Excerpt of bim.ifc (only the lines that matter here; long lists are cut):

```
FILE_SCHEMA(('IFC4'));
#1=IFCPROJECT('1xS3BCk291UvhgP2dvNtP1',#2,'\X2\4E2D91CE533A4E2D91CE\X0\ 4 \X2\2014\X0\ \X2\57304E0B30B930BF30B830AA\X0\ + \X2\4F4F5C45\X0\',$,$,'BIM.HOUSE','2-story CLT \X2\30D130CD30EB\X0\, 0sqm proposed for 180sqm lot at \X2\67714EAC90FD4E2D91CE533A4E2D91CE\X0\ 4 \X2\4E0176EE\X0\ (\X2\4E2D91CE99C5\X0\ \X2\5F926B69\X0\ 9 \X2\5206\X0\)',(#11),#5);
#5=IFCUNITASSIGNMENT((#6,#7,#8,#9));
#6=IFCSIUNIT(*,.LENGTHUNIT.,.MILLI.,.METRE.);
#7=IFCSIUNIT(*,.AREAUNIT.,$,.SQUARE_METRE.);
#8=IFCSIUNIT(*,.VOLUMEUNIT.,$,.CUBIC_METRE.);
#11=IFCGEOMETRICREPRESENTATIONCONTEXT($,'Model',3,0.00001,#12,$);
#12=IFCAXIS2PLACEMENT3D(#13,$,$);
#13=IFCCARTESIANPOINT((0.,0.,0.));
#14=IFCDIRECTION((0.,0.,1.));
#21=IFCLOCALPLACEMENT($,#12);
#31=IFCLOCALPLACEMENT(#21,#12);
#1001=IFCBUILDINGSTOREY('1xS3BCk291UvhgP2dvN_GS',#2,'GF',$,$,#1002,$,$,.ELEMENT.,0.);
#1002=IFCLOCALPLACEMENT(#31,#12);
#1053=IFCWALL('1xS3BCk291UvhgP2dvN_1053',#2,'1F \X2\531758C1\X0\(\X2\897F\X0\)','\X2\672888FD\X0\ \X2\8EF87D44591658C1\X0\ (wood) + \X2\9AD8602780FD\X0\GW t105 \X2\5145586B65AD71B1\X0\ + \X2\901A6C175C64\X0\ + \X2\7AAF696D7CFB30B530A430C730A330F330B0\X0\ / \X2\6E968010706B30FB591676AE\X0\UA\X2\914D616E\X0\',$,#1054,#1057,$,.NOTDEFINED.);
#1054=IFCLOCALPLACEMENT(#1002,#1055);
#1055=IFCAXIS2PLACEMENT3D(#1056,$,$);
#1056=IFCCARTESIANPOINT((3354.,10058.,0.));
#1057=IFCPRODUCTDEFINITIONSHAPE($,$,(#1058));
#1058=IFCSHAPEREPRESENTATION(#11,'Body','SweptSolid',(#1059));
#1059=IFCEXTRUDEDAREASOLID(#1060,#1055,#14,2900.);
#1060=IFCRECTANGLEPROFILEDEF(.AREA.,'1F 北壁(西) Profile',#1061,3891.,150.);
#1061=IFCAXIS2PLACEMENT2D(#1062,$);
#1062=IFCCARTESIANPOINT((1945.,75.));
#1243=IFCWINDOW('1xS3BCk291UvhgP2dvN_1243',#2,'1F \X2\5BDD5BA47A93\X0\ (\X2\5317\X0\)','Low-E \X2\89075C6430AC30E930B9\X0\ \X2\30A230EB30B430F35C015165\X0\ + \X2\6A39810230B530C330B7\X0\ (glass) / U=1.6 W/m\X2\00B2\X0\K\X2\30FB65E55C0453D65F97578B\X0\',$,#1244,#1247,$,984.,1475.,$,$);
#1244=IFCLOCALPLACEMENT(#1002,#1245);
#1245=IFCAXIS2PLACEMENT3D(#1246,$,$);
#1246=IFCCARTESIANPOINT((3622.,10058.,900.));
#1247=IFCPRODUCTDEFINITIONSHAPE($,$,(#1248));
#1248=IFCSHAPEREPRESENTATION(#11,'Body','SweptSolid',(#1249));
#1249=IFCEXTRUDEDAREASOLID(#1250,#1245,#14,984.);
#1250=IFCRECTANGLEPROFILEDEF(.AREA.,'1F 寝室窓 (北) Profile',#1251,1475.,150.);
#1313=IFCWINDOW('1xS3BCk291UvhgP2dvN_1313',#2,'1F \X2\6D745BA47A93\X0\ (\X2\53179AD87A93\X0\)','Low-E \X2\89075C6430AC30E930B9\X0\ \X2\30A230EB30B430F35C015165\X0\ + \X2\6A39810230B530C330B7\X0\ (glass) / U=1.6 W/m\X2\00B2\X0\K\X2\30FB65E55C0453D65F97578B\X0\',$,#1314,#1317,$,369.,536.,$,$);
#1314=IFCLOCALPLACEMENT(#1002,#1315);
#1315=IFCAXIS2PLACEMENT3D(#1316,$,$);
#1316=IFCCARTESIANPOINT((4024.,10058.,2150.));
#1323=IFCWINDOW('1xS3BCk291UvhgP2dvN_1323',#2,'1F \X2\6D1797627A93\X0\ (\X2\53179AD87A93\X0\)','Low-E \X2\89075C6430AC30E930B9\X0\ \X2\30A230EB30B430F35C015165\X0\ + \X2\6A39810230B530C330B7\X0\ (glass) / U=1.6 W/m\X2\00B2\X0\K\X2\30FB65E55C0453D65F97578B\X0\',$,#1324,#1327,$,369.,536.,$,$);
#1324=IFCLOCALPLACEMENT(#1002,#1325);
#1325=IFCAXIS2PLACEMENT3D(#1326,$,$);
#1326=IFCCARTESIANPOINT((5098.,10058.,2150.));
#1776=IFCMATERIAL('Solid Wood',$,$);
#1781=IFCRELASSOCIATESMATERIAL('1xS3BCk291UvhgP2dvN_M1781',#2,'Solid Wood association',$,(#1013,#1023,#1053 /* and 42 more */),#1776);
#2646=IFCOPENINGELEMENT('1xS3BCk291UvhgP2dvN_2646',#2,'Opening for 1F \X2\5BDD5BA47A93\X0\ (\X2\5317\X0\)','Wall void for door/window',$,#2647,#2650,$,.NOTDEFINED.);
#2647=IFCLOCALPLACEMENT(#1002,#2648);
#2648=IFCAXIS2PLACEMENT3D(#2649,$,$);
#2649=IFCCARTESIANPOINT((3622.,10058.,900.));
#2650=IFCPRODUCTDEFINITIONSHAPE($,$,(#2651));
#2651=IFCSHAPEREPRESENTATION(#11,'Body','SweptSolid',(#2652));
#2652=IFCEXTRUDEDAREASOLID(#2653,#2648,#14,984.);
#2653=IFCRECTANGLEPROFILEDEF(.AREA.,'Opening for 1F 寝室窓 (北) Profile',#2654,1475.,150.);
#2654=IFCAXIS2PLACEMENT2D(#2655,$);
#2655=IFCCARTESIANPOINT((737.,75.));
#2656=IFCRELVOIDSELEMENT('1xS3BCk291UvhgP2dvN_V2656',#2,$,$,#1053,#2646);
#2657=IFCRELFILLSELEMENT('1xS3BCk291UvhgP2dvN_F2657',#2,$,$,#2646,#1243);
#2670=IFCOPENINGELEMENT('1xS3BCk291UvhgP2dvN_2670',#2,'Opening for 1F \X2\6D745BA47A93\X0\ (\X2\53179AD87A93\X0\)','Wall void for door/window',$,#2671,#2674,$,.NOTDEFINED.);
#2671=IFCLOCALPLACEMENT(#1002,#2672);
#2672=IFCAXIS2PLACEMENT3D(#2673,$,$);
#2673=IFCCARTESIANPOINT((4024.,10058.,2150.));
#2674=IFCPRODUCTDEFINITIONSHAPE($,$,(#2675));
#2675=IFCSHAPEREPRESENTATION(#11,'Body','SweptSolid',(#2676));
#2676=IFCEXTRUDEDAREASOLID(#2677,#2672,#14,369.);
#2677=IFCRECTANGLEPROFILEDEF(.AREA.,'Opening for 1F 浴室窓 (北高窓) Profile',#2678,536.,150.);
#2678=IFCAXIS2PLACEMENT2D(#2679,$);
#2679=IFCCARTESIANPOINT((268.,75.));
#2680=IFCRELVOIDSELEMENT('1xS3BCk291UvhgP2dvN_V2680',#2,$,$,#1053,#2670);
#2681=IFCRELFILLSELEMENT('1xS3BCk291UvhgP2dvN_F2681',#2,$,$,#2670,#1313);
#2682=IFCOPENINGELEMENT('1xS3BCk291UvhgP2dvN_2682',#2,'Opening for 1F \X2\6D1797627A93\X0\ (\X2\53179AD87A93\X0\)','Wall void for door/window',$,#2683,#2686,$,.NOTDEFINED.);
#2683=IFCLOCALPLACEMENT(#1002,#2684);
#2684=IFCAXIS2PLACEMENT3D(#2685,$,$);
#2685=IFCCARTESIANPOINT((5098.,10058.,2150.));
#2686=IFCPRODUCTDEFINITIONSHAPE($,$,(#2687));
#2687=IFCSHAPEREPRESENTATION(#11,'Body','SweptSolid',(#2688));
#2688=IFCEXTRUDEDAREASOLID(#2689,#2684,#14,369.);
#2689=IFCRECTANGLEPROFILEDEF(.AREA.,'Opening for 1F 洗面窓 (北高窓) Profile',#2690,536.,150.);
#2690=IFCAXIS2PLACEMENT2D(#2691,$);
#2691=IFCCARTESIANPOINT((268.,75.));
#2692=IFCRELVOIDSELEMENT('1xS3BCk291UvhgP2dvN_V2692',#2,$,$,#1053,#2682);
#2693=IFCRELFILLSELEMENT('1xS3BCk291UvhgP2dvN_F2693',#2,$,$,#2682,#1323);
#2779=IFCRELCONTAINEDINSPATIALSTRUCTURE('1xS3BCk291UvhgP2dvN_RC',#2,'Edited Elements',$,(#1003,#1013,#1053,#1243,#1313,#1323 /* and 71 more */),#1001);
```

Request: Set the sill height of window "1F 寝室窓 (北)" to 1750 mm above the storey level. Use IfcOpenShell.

```python
import numpy as np
import ifcopenshell
import ifcopenshell.api.geometry
import ifcopenshell.geom
import ifcopenshell.util.element
import ifcopenshell.util.placement
import ifcopenshell.util.shape
import ifcopenshell.util.unit

model = ifcopenshell.open("bim.ifc")
unit_scale = ifcopenshell.util.unit.calculate_unit_scale(model)

window = model.by_id(1243)
opening = window.FillsVoids[0].RelatingOpeningElement
storey = ifcopenshell.util.element.get_container(window, ifc_class="IfcBuildingStorey")
level = ifcopenshell.util.placement.get_local_placement(storey.ObjectPlacement)[2, 3]

# The opening's origin need not be at the sill, so measure its lowest point.
shape = ifcopenshell.geom.create_shape(ifcopenshell.geom.settings(), opening)
bottom = ifcopenshell.util.shape.get_shape_bottom_elevation(shape, shape.geometry) / unit_scale
dz = level + 1.75 / unit_scale - bottom

shift = np.array([0.0, 0.0, dz])
# The window is not placed relative to its opening, so move both.
for product in (opening, window):
    matrix = ifcopenshell.util.placement.get_local_placement(product.ObjectPlacement)
    matrix[:3, 3] += shift
    ifcopenshell.api.geometry.edit_object_placement(model, product=product, matrix=matrix, is_si=False)

print(f"moved by {dz * unit_scale:+.3f} m")

model.write("bim_edited.ifc")
```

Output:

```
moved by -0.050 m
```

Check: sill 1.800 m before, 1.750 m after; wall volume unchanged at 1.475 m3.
